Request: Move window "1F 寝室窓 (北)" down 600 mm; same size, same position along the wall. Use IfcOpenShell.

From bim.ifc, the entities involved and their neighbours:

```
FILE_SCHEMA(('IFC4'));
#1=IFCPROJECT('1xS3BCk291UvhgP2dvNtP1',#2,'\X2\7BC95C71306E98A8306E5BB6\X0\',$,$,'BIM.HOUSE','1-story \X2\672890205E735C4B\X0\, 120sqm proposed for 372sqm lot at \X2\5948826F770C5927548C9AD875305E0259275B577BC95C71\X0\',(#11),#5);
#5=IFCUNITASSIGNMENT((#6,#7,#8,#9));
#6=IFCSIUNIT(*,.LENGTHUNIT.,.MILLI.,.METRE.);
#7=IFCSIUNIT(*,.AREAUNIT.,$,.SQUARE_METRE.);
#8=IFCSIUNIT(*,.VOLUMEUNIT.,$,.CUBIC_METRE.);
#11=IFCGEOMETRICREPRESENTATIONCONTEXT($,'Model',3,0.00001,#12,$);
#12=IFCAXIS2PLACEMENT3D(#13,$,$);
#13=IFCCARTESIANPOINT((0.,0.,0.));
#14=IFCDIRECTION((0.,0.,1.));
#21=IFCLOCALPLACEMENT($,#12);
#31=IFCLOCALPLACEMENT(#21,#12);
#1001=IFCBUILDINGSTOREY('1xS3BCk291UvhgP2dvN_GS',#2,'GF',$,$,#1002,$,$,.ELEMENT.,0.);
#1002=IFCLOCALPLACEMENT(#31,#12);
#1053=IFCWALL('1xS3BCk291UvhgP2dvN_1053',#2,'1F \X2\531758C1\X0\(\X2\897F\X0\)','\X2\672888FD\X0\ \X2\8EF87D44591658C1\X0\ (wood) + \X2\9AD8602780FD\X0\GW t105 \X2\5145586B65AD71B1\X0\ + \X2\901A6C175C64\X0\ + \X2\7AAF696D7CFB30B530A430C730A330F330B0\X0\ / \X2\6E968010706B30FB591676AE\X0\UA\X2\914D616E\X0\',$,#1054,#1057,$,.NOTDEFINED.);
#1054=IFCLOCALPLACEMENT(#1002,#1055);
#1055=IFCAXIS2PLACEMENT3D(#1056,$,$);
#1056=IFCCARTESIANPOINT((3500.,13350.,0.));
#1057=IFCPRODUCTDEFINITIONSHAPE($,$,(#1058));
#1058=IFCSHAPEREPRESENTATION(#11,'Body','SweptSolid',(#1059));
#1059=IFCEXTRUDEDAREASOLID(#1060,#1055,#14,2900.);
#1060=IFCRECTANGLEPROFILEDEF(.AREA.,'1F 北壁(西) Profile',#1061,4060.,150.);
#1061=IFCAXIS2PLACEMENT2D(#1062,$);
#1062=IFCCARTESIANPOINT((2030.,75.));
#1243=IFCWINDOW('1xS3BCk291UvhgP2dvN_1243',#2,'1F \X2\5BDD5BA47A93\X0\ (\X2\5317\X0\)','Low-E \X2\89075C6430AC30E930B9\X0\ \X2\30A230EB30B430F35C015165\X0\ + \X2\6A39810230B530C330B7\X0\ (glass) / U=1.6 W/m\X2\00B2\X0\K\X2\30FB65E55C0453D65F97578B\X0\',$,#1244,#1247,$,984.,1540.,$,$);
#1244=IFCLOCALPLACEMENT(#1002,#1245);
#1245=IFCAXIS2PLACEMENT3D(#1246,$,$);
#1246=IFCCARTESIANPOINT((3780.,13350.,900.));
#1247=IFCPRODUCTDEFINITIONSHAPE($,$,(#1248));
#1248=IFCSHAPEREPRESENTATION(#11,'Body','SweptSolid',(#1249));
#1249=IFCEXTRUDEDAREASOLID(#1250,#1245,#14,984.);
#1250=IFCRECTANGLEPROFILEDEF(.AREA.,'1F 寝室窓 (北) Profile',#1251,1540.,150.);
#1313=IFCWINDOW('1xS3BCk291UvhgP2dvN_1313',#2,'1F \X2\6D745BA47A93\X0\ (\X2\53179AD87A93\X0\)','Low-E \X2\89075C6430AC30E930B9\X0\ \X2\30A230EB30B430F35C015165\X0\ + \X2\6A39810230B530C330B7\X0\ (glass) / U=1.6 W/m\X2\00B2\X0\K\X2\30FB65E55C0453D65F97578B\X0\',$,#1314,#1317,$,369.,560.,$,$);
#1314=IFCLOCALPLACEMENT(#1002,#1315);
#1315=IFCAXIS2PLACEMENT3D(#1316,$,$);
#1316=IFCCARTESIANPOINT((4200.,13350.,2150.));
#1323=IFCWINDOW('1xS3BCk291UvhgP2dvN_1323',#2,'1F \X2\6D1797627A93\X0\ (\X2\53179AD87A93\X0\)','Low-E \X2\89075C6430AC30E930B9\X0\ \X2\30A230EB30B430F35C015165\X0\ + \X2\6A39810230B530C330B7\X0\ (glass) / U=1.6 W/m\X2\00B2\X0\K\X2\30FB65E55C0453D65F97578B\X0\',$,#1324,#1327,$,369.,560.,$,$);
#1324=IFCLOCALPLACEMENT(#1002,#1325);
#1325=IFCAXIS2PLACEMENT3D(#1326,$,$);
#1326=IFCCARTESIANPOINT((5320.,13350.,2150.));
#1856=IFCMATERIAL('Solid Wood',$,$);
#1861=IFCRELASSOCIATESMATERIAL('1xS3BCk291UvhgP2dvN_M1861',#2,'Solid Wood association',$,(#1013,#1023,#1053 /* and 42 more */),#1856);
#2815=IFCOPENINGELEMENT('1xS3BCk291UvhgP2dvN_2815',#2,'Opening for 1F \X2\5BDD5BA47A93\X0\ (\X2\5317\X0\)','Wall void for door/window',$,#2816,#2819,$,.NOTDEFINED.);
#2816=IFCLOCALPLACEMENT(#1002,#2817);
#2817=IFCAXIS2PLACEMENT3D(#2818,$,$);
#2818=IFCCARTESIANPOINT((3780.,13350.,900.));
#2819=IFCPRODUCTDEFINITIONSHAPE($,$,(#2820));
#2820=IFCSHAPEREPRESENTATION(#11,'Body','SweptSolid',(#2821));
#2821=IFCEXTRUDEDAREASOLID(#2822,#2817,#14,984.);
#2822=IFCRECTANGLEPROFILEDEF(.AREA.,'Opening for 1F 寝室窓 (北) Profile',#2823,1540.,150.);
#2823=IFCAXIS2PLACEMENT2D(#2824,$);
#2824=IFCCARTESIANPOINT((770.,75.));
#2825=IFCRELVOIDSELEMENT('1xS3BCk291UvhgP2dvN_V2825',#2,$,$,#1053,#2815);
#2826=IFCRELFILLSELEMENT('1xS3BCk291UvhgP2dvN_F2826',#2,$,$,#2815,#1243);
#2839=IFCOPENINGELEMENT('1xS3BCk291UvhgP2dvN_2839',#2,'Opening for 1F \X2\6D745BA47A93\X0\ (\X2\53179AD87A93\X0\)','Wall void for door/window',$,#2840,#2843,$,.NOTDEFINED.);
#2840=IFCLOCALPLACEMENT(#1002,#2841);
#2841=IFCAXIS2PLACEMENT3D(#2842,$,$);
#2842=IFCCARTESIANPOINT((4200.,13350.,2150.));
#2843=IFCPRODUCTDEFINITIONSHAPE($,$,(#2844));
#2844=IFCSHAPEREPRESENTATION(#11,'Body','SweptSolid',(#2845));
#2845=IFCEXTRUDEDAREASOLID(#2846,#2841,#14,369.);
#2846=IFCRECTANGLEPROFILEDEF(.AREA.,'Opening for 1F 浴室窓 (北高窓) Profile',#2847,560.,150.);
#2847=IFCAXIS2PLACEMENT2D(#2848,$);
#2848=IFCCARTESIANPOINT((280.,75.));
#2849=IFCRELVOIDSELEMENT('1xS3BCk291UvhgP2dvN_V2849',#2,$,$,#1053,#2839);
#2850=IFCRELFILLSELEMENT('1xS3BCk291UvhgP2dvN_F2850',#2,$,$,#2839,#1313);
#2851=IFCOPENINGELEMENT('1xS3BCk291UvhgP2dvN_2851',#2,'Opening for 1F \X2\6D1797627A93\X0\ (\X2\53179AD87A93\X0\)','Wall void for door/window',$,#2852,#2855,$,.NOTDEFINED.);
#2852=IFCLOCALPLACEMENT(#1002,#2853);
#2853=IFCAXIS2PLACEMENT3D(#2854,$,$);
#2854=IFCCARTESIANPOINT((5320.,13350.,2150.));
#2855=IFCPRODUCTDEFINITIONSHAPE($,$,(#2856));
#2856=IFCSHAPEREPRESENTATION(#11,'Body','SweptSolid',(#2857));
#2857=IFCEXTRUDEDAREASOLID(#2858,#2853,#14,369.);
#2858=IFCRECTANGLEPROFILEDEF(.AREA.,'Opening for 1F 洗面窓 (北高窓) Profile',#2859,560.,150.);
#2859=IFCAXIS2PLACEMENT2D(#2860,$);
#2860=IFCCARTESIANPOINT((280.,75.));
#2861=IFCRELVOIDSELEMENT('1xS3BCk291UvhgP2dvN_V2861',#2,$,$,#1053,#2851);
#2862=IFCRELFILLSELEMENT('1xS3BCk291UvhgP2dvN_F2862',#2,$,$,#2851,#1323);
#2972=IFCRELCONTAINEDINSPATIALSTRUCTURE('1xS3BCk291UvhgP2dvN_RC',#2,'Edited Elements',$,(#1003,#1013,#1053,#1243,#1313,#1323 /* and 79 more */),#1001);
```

```python
import numpy as np
import ifcopenshell
import ifcopenshell.api.geometry
import ifcopenshell.util.placement
import ifcopenshell.util.unit

model = ifcopenshell.open("bim.ifc")
unit_scale = ifcopenshell.util.unit.calculate_unit_scale(model)

window = model.by_id(1243)
opening = window.FillsVoids[0].RelatingOpeningElement
dz = -0.6 / unit_scale

shift = np.array([0.0, 0.0, dz])
# The window is not placed relative to its opening, so move both.
for product in (opening, window):
    matrix = ifcopenshell.util.placement.get_local_placement(product.ObjectPlacement)
    matrix[:3, 3] += shift
    ifcopenshell.api.geometry.edit_object_placement(model, product=product, matrix=matrix, is_si=False)

print(f"moved by {dz * unit_scale:+.3f} m")

model.write("bim_v2.ifc")
```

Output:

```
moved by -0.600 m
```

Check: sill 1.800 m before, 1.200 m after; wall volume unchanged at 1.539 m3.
